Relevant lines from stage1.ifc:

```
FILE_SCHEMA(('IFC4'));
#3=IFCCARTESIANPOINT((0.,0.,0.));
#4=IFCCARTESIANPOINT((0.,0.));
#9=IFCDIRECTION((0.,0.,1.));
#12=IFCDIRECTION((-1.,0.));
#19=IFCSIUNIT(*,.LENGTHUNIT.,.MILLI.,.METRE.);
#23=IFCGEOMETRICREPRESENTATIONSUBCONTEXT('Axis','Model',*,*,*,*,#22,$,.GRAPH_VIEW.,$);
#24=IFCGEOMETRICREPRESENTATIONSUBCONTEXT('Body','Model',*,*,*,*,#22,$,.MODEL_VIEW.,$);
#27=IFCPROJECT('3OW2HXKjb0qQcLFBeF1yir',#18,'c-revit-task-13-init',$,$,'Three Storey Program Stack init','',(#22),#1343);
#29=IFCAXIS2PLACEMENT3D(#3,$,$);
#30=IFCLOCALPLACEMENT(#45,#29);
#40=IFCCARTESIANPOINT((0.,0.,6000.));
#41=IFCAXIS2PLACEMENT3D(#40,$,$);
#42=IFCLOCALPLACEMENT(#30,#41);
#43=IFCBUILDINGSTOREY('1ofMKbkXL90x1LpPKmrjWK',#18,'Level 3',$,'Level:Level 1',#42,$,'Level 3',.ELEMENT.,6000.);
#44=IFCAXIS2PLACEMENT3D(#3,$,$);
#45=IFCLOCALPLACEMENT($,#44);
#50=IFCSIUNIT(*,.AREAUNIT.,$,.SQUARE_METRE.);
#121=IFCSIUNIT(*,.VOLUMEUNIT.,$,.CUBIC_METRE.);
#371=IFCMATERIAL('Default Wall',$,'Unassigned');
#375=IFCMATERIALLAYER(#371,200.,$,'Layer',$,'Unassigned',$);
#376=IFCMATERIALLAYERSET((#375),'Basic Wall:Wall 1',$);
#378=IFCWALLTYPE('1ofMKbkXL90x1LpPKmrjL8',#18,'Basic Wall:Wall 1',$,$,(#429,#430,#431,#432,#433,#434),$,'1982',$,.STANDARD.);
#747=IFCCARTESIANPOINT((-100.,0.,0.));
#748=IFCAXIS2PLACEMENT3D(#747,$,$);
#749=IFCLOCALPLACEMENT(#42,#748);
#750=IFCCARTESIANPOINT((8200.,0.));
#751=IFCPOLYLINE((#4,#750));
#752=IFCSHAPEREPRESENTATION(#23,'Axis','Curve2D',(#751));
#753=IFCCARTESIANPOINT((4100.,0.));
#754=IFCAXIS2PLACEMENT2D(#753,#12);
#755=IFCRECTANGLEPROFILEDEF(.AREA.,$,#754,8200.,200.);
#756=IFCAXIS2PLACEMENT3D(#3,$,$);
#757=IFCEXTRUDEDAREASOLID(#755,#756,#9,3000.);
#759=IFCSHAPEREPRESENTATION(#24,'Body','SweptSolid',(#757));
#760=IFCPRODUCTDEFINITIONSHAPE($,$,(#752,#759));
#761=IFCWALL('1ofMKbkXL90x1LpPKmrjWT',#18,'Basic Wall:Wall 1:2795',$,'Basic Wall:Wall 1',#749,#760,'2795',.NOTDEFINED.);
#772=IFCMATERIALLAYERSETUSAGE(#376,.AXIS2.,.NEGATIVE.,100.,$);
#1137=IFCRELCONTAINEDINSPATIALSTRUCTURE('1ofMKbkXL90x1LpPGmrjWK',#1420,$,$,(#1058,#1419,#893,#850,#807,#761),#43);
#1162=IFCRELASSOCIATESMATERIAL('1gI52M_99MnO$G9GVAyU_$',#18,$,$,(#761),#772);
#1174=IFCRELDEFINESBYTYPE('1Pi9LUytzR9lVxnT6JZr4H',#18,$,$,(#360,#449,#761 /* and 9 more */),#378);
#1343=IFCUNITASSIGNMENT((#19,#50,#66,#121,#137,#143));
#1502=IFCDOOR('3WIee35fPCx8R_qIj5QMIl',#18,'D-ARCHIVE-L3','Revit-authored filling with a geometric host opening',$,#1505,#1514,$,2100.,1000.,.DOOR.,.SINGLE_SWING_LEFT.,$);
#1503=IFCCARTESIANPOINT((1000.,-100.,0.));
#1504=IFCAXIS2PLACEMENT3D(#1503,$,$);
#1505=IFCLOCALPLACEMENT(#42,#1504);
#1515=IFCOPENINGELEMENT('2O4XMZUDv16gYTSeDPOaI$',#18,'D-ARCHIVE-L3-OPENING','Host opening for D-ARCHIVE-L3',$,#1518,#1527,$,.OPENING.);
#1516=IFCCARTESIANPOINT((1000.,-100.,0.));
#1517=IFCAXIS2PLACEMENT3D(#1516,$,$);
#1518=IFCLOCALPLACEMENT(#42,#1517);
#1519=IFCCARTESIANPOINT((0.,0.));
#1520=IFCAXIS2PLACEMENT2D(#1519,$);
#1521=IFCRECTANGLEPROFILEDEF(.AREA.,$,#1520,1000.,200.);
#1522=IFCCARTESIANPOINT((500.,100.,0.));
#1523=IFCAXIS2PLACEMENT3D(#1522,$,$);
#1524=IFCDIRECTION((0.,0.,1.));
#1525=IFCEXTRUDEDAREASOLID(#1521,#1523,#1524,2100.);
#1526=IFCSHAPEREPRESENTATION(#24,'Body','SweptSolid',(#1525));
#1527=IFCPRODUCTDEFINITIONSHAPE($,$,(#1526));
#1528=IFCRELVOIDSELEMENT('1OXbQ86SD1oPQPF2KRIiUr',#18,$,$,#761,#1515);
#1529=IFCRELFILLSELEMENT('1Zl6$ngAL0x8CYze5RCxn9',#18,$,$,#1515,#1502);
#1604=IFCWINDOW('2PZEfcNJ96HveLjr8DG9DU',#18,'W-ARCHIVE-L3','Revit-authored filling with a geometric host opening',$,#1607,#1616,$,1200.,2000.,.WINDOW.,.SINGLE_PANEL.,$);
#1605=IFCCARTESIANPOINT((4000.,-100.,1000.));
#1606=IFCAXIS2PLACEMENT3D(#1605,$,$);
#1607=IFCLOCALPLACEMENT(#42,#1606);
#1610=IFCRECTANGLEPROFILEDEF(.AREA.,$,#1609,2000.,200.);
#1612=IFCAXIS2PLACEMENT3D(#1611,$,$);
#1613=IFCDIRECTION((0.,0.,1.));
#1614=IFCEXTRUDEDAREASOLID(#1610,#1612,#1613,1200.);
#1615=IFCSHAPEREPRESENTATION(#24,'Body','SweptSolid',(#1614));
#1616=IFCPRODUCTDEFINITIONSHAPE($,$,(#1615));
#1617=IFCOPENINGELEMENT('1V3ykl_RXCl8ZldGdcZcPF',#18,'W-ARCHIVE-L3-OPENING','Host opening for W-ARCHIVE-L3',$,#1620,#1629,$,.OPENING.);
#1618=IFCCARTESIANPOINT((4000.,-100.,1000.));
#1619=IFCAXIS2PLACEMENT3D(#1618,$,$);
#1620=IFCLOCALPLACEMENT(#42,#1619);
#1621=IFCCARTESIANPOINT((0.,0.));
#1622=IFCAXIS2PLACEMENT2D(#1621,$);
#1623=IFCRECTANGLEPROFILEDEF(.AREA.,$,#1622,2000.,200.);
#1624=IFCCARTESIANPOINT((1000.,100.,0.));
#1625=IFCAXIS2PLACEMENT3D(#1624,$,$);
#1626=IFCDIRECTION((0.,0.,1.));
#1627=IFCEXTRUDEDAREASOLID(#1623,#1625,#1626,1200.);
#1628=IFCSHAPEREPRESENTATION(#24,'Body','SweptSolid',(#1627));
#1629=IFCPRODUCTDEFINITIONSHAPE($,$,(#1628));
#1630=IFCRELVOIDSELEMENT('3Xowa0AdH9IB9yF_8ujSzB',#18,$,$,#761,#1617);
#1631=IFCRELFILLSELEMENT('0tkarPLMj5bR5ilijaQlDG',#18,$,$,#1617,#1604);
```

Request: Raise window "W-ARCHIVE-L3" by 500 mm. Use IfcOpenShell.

```python
import numpy as np
import ifcopenshell
import ifcopenshell.api.geometry
import ifcopenshell.util.placement
import ifcopenshell.util.unit

model = ifcopenshell.open("stage1.ifc")
unit_scale = ifcopenshell.util.unit.calculate_unit_scale(model)

window = model.by_guid("2PZEfcNJ96HveLjr8DG9DU")
opening = window.FillsVoids[0].RelatingOpeningElement
dz = 0.5 / unit_scale

shift = np.array([0.0, 0.0, dz])
# The window is not placed relative to its opening, so move both.
for product in (opening, window):
    matrix = ifcopenshell.util.placement.get_local_placement(product.ObjectPlacement)
    matrix[:3, 3] += shift
    ifcopenshell.api.geometry.edit_object_placement(model, product=product, matrix=matrix, is_si=False)

print(f"moved by {dz * unit_scale:+.3f} m")

model.write("stage1-out.ifc")
```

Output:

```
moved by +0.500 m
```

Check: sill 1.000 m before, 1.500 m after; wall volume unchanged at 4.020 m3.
